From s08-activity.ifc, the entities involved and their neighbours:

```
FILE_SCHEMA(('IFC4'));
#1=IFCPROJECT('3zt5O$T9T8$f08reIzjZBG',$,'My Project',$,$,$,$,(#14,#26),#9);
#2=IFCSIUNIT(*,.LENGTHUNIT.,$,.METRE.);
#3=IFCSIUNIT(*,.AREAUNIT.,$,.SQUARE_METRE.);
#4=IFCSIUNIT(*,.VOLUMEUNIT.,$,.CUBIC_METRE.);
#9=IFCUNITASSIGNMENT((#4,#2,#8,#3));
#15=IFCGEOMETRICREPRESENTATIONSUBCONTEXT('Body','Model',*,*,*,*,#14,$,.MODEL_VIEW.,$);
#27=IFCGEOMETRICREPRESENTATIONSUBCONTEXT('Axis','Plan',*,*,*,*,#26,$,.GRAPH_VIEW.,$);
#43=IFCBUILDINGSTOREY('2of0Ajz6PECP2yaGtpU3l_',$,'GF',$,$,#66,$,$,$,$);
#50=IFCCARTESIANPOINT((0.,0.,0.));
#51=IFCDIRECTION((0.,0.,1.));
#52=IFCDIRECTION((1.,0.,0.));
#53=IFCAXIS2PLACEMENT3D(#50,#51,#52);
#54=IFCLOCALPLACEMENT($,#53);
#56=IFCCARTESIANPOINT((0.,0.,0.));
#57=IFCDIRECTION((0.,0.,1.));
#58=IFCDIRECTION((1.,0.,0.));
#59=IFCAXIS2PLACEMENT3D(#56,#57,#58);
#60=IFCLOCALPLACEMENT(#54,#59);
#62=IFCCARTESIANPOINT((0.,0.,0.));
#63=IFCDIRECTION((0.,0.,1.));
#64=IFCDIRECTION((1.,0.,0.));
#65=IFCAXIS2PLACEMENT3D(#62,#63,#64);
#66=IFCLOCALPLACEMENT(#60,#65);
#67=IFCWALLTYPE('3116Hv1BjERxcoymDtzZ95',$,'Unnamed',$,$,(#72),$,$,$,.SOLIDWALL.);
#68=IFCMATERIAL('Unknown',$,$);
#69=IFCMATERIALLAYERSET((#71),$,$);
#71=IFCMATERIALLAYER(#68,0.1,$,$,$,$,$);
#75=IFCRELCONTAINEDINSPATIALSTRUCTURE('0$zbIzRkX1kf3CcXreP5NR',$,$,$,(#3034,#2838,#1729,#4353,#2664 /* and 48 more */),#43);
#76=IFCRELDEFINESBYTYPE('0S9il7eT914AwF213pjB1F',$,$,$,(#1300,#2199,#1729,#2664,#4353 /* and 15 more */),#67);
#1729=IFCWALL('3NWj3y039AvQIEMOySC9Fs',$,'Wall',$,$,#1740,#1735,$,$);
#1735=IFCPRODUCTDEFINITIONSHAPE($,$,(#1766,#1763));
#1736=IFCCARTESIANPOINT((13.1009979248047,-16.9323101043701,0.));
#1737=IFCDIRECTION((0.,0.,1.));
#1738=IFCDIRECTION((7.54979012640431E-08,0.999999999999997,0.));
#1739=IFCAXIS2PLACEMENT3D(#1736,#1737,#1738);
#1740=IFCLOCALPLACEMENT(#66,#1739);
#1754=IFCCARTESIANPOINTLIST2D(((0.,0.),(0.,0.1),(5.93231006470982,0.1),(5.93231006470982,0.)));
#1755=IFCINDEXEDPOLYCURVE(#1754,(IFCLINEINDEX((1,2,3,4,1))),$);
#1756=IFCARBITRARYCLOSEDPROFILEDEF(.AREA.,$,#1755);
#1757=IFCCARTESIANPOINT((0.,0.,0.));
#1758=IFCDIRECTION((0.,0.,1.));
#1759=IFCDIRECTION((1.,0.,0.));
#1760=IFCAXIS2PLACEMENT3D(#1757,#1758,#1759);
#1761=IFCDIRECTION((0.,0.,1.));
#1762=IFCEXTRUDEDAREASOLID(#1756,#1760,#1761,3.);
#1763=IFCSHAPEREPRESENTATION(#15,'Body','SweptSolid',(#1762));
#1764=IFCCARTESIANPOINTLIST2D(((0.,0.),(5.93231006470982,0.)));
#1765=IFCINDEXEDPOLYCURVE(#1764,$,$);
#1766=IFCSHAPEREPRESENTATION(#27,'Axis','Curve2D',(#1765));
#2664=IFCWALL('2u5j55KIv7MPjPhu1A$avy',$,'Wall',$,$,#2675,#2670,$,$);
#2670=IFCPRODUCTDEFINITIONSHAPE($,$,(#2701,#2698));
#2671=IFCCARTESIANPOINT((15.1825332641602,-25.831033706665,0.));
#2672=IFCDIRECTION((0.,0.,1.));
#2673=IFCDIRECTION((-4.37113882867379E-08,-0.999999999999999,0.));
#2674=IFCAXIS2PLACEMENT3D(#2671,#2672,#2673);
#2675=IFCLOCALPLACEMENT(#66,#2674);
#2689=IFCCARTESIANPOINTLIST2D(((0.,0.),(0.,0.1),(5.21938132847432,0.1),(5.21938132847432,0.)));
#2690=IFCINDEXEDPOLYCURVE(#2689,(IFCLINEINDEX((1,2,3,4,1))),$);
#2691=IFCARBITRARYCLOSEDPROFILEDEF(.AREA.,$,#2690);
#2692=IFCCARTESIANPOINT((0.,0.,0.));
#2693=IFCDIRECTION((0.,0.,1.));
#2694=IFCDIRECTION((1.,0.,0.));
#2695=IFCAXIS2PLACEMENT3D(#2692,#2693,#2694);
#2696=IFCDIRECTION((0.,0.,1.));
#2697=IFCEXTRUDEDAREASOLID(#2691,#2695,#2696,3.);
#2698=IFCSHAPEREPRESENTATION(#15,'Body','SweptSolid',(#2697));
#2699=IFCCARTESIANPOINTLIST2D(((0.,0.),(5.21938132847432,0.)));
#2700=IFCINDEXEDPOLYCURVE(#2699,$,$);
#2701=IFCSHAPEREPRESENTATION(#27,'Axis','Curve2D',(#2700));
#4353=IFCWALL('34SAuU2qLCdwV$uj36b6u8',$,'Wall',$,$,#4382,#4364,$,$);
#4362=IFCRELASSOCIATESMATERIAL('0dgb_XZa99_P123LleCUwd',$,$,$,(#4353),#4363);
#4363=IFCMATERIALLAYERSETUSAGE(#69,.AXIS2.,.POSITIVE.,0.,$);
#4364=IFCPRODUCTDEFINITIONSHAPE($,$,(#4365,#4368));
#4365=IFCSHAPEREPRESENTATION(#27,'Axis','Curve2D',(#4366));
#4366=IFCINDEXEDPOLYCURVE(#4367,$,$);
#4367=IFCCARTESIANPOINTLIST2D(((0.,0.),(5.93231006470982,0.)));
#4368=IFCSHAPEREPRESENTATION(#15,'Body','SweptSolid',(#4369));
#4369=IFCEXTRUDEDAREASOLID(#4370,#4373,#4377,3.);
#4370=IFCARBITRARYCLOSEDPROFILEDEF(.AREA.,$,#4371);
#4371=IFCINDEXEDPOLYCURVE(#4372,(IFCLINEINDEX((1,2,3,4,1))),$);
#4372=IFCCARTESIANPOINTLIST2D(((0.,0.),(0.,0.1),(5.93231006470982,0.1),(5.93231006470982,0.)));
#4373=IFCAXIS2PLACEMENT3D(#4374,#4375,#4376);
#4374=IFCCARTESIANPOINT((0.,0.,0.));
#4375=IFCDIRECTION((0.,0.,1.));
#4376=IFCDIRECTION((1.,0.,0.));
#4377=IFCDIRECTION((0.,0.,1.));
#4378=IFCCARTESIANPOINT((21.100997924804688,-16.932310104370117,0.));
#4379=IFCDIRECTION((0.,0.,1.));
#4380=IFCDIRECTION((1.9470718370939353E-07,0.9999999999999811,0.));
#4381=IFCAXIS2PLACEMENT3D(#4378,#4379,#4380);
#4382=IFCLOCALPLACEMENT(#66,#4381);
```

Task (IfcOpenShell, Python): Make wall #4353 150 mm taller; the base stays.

```python
import ifcopenshell
import ifcopenshell.geom
import ifcopenshell.util.representation
import ifcopenshell.util.shape

model = ifcopenshell.open("s08-activity.ifc")
settings = ifcopenshell.geom.settings()


def volume(element):
    """Net volume in cubic metres, openings subtracted."""
    shape = ifcopenshell.geom.create_shape(settings, element)
    return ifcopenshell.util.shape.get_volume(shape.geometry)


wall = model.by_guid("34SAuU2qLCdwV$uj36b6u8")
before = volume(wall)

body = ifcopenshell.util.representation.get_representation(wall, "Model", "Body")
solid = body.Items[0]
old_height = solid.Depth
solid.Depth += 0.15
after = volume(wall)

print(f"height {old_height:g} -> {solid.Depth:g}, volume {before:.3f} -> {after:.3f} m3")

model.write("s08-activity_updated.ifc")
```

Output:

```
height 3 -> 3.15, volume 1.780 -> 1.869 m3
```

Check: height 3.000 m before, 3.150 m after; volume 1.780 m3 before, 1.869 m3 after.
